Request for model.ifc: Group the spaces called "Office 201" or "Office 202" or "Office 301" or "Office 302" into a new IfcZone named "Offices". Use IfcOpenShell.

First a look at what the model holds.

```python
import ifcopenshell

model = ifcopenshell.open("model.ifc")
print(model.schema)
seen = {}
for space in model.by_type("IfcSpace"):
    seen[space.Name] = seen.get(space.Name, 0) + 1
for name, count in sorted(seen.items(), key=str):
    print(count, "x", name)
print("zones:", [z.Name for z in model.by_type("IfcZone")][:20])
```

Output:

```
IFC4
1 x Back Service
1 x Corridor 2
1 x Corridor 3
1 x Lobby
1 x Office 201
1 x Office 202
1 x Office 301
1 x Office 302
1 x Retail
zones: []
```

```python
import ifcopenshell
import ifcopenshell.api.group
import ifcopenshell.api.root

model = ifcopenshell.open("model.ifc")

names = {"Office 201", "Office 202", "Office 301", "Office 302"}
spaces = [s for s in model.by_type("IfcSpace") if s.Name in names]

zone = ifcopenshell.api.root.create_entity(model, ifc_class="IfcZone", name="Offices")
ifcopenshell.api.group.assign_group(model, products=spaces, group=zone)
print(len(spaces), "spaces in", zone.Name)

model.write("model_edited.ifc")
```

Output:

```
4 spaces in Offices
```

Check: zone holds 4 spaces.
